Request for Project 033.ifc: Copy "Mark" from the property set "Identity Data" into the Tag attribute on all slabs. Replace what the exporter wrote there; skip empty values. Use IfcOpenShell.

First a look at what the model holds.

```python
import ifcopenshell
import ifcopenshell.util.element

model = ifcopenshell.open("Project 033.ifc")
print(model.schema)
slabs = model.by_type("IfcSlab")
print(len(slabs), "slabs")
for e in slabs[:8]:
    source = ifcopenshell.util.element.get_pset(e, "Identity Data", "Mark")
    target = e.Tag
    print(e.id(), repr(source), repr(target), sep=" | ")
```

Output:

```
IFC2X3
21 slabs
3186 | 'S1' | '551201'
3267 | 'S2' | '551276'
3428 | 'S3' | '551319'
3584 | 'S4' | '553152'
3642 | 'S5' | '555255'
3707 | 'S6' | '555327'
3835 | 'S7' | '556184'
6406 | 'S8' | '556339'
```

```python
import ifcopenshell
import ifcopenshell.util.element

model = ifcopenshell.open("Project 033.ifc")

count = 0
for e in model.by_type("IfcSlab"):
    value = ifcopenshell.util.element.get_pset(e, "Identity Data", "Mark")
    current = e.Tag
    if not value or not value.strip() or current == value:
        continue
    e.Tag = value
    count += 1

print(count, "slabs updated")

model.write("Project 033-out.ifc")
```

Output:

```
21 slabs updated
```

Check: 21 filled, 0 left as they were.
